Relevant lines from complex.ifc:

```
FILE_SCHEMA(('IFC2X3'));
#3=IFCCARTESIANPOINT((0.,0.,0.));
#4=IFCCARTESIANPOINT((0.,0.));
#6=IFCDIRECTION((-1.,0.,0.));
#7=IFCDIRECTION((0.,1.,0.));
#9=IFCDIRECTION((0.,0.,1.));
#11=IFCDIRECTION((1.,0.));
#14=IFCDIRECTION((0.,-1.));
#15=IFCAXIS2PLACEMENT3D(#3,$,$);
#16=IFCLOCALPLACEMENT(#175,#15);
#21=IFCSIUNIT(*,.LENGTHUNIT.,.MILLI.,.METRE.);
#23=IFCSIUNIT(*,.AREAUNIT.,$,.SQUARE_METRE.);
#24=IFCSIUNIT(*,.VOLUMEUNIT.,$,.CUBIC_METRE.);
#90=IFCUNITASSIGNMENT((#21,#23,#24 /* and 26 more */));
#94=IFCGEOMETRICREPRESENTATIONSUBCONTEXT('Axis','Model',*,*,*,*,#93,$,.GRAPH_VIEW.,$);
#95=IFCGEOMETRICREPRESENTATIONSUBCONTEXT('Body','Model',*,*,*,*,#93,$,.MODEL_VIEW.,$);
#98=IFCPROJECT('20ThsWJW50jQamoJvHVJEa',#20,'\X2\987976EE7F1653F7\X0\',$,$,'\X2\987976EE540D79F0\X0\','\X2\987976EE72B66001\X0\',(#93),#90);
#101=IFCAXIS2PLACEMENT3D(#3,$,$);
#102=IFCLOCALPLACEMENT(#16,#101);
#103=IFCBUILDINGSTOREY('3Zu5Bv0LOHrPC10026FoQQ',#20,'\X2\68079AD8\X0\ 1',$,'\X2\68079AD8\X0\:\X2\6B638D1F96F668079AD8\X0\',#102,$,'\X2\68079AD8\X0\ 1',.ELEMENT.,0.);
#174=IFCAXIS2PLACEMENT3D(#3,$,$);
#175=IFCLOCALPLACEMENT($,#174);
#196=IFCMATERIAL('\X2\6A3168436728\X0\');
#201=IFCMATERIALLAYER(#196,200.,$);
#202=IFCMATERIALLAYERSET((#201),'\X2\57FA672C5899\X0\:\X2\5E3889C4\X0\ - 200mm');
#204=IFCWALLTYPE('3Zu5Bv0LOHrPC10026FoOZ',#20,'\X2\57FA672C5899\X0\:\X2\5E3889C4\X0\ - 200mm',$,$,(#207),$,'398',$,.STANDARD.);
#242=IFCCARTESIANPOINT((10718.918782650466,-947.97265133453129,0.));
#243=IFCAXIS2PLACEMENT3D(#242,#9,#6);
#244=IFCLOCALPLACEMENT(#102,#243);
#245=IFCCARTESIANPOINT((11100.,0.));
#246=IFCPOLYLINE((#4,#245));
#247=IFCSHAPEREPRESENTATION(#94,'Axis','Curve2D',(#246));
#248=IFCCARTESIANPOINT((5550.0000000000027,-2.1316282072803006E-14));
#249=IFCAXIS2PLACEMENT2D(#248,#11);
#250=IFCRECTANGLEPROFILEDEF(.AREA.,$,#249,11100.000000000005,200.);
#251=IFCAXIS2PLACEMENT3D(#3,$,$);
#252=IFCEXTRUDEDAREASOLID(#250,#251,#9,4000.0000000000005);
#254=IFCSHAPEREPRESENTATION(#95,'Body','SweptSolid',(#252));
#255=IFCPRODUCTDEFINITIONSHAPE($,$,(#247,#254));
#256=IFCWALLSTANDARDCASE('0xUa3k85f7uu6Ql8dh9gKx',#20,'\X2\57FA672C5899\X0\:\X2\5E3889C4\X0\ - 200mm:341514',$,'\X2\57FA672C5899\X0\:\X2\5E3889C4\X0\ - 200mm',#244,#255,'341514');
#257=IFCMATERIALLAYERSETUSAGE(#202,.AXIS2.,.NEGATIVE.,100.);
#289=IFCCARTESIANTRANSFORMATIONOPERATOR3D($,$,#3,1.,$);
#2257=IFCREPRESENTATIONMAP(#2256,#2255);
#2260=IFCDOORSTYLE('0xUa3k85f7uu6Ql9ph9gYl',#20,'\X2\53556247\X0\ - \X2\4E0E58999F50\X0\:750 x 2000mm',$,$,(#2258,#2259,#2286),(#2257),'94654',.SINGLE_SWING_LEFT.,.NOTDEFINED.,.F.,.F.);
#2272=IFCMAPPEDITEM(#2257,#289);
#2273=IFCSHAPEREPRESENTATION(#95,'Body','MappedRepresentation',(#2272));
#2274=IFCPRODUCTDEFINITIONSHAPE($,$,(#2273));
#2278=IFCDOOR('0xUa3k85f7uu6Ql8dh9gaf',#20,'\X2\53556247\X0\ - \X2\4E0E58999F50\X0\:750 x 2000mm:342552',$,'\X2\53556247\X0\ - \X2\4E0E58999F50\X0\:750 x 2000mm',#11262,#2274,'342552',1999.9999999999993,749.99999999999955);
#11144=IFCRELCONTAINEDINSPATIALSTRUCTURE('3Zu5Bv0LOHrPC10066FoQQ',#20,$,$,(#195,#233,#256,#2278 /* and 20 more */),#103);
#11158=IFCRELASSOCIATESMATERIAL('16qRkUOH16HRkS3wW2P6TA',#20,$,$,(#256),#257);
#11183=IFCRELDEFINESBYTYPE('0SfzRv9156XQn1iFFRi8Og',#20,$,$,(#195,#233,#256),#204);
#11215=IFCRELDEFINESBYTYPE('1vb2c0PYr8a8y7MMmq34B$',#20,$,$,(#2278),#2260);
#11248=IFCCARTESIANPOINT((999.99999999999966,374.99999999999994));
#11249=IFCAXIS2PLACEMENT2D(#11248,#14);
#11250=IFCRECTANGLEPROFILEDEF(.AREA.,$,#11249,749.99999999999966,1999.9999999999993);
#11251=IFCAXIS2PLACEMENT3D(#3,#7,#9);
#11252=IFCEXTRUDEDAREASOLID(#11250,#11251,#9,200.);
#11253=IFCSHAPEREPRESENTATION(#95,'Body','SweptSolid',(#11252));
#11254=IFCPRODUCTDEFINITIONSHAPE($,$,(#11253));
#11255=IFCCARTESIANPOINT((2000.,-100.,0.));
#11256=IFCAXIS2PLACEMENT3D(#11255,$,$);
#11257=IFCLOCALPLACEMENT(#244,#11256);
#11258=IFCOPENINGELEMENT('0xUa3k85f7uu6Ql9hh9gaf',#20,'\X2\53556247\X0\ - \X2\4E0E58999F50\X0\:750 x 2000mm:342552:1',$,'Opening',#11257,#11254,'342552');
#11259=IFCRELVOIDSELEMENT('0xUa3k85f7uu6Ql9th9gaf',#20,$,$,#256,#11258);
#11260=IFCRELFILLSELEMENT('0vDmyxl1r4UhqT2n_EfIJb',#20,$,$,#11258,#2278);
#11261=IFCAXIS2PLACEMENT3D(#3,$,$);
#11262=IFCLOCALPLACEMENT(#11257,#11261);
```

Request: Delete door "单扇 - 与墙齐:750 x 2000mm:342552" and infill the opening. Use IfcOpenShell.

```python
import ifcopenshell
import ifcopenshell.api.feature
import ifcopenshell.api.root
import ifcopenshell.geom
import ifcopenshell.util.shape

model = ifcopenshell.open("complex.ifc")
settings = ifcopenshell.geom.settings()


def volume(element):
    """Net volume in cubic metres, openings subtracted."""
    shape = ifcopenshell.geom.create_shape(settings, element)
    return ifcopenshell.util.shape.get_volume(shape.geometry)


door = model.by_guid("0xUa3k85f7uu6Ql8dh9gaf")
opening = door.FillsVoids[0].RelatingOpeningElement
wall = opening.VoidsElements[0].RelatingBuildingElement
before = volume(wall)

ifcopenshell.api.root.remove_product(model, product=door)
ifcopenshell.api.feature.remove_feature(model, feature=opening)

after = volume(wall)

print(f"wall volume {before:.3f} -> {after:.3f} m3")

model.write("complex_updated.ifc")
```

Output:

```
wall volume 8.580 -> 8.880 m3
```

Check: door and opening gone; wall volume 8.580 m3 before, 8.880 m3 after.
